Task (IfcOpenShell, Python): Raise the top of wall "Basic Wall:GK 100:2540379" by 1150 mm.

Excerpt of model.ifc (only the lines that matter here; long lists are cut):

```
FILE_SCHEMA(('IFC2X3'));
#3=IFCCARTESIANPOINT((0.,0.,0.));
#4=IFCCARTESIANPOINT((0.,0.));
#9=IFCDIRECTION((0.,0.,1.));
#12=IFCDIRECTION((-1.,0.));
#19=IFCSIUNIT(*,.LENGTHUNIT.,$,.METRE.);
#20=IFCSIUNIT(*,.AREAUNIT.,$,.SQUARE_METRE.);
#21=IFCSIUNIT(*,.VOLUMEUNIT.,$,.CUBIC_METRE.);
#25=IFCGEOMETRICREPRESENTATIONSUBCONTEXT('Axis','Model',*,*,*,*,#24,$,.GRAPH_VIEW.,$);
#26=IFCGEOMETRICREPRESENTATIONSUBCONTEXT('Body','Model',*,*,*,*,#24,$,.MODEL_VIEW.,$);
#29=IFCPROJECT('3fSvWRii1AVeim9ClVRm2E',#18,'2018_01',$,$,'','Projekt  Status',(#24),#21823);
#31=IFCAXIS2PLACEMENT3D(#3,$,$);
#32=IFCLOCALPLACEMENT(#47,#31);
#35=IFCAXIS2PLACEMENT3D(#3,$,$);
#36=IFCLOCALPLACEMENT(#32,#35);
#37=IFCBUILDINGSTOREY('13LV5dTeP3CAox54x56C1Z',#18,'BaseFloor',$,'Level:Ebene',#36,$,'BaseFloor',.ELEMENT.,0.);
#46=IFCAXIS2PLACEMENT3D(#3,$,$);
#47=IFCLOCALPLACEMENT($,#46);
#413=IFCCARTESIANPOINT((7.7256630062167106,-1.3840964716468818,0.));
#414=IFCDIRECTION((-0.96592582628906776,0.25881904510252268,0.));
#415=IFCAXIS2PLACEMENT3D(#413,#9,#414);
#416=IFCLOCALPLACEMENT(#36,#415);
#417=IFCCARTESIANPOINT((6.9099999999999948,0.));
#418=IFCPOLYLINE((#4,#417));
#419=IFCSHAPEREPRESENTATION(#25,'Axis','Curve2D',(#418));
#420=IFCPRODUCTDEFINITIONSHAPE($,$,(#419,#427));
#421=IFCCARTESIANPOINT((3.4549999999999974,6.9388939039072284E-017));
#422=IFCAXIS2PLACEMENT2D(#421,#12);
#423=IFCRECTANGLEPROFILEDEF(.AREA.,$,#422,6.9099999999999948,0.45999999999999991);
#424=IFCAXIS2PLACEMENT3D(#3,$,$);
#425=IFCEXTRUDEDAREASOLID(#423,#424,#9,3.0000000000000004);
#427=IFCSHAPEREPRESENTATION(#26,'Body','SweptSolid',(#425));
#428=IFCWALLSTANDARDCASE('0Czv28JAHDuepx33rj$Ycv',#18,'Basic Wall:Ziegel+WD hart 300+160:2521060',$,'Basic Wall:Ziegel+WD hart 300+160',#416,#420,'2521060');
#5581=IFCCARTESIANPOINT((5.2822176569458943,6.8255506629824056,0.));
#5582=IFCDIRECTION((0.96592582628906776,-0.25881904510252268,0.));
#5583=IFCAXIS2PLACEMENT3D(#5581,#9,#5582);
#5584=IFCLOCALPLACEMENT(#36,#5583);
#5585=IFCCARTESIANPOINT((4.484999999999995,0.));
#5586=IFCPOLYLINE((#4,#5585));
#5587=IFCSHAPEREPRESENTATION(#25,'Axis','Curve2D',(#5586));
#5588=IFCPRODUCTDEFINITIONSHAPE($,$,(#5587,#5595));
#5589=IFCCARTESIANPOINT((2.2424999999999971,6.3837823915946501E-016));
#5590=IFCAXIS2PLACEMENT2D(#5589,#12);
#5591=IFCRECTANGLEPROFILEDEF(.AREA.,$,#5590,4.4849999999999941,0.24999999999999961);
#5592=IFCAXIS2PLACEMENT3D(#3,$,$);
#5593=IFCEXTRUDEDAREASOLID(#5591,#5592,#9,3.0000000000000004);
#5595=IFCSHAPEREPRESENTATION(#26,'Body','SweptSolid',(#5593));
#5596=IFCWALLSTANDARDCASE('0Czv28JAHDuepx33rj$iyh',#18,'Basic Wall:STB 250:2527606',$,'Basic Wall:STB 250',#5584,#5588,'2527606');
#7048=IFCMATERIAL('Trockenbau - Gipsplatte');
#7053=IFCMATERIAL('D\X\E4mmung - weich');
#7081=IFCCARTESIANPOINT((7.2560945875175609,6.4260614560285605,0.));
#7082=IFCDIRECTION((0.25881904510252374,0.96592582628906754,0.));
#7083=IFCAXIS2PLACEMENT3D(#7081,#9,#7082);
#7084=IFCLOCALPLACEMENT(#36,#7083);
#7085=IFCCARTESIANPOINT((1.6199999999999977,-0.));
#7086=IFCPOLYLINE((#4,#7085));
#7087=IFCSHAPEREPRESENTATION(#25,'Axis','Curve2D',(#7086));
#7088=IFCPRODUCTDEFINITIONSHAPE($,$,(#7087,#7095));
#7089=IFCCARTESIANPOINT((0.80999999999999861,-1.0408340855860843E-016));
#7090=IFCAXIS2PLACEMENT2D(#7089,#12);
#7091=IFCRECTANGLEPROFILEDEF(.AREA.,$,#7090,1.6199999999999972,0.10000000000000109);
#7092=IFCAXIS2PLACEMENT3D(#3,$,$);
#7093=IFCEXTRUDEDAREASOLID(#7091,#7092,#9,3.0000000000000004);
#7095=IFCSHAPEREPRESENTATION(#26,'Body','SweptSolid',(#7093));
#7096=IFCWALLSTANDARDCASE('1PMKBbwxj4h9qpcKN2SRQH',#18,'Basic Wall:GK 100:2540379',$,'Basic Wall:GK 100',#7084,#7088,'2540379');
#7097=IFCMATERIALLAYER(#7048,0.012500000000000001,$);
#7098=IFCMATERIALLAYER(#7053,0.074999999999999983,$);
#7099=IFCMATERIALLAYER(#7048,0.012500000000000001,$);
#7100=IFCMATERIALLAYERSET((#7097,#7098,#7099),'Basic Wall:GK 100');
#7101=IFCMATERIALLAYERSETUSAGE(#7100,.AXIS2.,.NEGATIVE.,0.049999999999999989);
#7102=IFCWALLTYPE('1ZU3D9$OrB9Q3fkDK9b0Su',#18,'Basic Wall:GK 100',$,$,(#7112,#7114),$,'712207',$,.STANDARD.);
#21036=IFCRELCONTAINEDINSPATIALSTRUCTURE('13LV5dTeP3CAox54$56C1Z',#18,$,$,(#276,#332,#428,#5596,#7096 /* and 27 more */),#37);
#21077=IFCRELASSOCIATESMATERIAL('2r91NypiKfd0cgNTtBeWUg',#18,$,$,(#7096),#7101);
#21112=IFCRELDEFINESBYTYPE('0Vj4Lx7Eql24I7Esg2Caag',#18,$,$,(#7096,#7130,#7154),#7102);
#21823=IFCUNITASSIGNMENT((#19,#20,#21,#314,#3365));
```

```python
import ifcopenshell
import ifcopenshell.geom
import ifcopenshell.util.representation
import ifcopenshell.util.shape

model = ifcopenshell.open("model.ifc")
settings = ifcopenshell.geom.settings()


def volume(element):
    """Net volume in cubic metres, openings subtracted."""
    shape = ifcopenshell.geom.create_shape(settings, element)
    return ifcopenshell.util.shape.get_volume(shape.geometry)


wall = model.by_guid("1PMKBbwxj4h9qpcKN2SRQH")
before = volume(wall)

body = ifcopenshell.util.representation.get_representation(wall, "Model", "Body")
solid = body.Items[0]
old_height = solid.Depth
solid.Depth += 1.15
after = volume(wall)

print(f"height {old_height:g} -> {solid.Depth:g}, volume {before:.3f} -> {after:.3f} m3")

model.write("model_updated.ifc")
```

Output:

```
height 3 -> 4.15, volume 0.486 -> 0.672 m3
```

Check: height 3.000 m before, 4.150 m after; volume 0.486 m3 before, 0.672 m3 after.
